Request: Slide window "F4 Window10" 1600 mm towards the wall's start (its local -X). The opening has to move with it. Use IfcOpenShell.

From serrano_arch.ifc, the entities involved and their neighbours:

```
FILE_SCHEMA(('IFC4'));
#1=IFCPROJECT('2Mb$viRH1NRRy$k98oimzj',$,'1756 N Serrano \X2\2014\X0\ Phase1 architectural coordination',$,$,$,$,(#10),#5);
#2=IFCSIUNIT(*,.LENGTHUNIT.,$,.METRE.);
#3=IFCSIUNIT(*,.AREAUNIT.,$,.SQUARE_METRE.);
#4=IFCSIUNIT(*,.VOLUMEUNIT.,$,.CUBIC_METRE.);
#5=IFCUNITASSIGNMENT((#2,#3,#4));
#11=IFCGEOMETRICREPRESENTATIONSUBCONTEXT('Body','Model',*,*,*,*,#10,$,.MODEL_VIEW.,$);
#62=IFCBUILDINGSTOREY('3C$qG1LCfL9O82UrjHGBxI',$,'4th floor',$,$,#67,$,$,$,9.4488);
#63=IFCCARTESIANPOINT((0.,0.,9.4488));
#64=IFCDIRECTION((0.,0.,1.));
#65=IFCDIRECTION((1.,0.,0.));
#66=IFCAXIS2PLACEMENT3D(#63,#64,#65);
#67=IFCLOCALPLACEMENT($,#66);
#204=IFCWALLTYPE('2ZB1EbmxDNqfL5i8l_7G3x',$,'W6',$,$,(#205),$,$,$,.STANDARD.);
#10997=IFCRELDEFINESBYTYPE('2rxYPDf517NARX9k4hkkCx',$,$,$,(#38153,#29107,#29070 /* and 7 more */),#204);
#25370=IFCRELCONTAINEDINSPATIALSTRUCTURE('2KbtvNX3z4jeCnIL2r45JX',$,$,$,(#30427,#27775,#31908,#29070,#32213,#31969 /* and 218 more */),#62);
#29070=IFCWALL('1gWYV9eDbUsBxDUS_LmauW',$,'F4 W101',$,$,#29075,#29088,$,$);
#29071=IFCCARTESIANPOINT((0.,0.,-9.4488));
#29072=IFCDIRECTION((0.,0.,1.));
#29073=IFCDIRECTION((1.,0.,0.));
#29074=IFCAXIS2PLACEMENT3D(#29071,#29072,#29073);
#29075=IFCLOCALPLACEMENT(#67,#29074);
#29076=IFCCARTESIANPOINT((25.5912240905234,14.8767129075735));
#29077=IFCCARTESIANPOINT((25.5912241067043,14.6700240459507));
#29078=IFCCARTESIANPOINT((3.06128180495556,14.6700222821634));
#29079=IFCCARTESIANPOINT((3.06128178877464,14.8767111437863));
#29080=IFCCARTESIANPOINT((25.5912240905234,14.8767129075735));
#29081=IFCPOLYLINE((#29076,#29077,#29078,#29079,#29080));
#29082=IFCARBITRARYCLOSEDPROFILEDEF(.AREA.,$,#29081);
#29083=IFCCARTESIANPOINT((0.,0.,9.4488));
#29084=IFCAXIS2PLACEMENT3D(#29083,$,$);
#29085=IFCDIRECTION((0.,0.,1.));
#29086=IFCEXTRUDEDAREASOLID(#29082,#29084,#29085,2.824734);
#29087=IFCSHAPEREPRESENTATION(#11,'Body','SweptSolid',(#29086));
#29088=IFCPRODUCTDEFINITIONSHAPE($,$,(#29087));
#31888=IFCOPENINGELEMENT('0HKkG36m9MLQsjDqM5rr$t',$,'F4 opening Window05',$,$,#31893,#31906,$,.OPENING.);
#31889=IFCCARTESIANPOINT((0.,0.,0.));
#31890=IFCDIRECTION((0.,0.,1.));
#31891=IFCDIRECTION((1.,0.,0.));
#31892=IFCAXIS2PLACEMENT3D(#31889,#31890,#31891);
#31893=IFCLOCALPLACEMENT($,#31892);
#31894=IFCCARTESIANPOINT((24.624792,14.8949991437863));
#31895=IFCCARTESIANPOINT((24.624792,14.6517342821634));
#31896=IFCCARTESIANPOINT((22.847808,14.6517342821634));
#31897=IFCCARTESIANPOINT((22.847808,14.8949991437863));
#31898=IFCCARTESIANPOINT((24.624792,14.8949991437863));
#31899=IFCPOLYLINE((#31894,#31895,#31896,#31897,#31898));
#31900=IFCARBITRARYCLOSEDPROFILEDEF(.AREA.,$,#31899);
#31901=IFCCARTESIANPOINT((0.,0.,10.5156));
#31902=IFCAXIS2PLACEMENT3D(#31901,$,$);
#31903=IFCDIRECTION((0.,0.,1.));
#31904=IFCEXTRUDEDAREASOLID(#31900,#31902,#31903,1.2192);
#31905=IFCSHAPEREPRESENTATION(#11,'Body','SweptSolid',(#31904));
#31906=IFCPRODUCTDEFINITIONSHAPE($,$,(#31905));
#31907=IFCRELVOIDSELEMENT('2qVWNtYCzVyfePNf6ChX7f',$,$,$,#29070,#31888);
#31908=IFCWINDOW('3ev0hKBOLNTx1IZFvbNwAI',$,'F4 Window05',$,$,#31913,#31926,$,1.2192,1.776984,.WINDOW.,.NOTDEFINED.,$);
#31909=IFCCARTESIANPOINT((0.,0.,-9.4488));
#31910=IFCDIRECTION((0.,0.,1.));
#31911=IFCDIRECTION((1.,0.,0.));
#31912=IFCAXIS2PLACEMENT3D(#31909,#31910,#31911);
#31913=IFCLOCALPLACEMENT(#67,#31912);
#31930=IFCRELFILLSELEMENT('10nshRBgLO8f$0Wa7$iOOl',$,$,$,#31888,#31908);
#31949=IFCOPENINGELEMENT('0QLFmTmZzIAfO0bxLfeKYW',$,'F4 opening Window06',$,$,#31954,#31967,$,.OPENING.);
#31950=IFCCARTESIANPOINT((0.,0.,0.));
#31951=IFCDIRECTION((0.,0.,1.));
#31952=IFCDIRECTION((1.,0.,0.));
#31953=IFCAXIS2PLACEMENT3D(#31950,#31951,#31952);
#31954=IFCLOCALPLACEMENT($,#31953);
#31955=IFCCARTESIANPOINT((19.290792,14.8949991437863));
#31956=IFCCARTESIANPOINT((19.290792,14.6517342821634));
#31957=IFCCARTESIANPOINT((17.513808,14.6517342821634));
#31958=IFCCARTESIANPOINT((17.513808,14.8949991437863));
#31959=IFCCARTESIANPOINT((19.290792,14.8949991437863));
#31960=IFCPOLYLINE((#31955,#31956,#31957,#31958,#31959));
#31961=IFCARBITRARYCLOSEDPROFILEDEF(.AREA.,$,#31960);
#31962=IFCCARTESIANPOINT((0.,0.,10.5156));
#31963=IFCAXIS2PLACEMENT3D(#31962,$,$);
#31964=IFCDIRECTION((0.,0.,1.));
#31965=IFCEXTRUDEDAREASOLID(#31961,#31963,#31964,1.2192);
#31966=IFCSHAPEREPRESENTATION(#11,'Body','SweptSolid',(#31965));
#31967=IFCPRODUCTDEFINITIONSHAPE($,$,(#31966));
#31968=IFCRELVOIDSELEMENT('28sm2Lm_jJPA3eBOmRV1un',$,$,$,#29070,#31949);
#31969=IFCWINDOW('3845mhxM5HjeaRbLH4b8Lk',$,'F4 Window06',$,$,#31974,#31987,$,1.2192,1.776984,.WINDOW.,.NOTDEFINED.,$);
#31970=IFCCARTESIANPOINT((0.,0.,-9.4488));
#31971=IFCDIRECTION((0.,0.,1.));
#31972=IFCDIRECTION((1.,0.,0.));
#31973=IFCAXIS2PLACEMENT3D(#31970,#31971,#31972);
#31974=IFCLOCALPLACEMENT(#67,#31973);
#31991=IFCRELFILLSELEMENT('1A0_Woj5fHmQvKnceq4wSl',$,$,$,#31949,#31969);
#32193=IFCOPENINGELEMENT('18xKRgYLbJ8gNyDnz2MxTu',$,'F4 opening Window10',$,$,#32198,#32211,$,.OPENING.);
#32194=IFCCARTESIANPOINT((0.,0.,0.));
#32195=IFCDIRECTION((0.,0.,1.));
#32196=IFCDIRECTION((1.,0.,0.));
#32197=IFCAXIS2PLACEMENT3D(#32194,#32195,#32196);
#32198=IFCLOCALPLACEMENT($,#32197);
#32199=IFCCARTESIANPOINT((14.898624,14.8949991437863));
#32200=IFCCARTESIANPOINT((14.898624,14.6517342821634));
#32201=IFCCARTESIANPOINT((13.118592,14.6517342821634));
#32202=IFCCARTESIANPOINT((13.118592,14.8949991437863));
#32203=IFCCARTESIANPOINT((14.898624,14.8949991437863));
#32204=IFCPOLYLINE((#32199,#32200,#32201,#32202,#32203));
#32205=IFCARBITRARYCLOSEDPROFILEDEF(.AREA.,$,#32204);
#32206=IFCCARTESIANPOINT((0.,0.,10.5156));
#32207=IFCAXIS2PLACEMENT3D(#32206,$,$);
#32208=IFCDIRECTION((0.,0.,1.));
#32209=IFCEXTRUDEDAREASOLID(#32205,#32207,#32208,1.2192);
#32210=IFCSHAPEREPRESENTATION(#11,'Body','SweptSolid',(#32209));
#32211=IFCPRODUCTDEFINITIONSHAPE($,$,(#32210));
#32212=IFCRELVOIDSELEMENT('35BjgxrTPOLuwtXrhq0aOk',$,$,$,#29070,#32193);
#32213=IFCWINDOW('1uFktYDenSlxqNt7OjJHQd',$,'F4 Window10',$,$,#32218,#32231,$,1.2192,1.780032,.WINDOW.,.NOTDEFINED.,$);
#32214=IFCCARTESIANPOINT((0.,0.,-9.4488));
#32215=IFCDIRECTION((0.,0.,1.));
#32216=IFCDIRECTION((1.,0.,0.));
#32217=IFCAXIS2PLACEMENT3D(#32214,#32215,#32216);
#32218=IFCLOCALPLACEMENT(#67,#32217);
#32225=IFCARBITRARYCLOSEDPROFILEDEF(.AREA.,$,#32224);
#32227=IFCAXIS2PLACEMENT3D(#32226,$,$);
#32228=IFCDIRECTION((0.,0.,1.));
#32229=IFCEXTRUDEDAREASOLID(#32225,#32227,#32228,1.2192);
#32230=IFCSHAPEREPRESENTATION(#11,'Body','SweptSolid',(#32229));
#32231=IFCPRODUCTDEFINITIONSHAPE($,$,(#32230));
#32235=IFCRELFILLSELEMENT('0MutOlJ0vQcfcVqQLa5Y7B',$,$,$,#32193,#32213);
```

```python
import ifcopenshell
import ifcopenshell.api.geometry
import ifcopenshell.util.placement
import ifcopenshell.util.unit

model = ifcopenshell.open("serrano_arch.ifc")
unit_scale = ifcopenshell.util.unit.calculate_unit_scale(model)

window = model.by_guid("1uFktYDenSlxqNt7OjJHQd")
opening = window.FillsVoids[0].RelatingOpeningElement
wall = opening.VoidsElements[0].RelatingBuildingElement

wall_matrix = ifcopenshell.util.placement.get_local_placement(wall.ObjectPlacement)
shift = wall_matrix[:3, 0] * -1.6 / unit_scale
before = ifcopenshell.util.placement.get_local_placement(window.ObjectPlacement)[:3, 3].copy()

# The window is not placed relative to its opening, so move both.
for product in (opening, window):
    matrix = ifcopenshell.util.placement.get_local_placement(product.ObjectPlacement)
    matrix[:3, 3] += shift
    ifcopenshell.api.geometry.edit_object_placement(model, product=product, matrix=matrix, is_si=False)

after = ifcopenshell.util.placement.get_local_placement(window.ObjectPlacement)[:3, 3]
print("window moved by", (after - before).round(3) + 0.0)

model.write("serrano_arch-out.ifc")
```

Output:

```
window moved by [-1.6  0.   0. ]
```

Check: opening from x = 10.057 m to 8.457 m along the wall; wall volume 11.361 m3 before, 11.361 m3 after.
